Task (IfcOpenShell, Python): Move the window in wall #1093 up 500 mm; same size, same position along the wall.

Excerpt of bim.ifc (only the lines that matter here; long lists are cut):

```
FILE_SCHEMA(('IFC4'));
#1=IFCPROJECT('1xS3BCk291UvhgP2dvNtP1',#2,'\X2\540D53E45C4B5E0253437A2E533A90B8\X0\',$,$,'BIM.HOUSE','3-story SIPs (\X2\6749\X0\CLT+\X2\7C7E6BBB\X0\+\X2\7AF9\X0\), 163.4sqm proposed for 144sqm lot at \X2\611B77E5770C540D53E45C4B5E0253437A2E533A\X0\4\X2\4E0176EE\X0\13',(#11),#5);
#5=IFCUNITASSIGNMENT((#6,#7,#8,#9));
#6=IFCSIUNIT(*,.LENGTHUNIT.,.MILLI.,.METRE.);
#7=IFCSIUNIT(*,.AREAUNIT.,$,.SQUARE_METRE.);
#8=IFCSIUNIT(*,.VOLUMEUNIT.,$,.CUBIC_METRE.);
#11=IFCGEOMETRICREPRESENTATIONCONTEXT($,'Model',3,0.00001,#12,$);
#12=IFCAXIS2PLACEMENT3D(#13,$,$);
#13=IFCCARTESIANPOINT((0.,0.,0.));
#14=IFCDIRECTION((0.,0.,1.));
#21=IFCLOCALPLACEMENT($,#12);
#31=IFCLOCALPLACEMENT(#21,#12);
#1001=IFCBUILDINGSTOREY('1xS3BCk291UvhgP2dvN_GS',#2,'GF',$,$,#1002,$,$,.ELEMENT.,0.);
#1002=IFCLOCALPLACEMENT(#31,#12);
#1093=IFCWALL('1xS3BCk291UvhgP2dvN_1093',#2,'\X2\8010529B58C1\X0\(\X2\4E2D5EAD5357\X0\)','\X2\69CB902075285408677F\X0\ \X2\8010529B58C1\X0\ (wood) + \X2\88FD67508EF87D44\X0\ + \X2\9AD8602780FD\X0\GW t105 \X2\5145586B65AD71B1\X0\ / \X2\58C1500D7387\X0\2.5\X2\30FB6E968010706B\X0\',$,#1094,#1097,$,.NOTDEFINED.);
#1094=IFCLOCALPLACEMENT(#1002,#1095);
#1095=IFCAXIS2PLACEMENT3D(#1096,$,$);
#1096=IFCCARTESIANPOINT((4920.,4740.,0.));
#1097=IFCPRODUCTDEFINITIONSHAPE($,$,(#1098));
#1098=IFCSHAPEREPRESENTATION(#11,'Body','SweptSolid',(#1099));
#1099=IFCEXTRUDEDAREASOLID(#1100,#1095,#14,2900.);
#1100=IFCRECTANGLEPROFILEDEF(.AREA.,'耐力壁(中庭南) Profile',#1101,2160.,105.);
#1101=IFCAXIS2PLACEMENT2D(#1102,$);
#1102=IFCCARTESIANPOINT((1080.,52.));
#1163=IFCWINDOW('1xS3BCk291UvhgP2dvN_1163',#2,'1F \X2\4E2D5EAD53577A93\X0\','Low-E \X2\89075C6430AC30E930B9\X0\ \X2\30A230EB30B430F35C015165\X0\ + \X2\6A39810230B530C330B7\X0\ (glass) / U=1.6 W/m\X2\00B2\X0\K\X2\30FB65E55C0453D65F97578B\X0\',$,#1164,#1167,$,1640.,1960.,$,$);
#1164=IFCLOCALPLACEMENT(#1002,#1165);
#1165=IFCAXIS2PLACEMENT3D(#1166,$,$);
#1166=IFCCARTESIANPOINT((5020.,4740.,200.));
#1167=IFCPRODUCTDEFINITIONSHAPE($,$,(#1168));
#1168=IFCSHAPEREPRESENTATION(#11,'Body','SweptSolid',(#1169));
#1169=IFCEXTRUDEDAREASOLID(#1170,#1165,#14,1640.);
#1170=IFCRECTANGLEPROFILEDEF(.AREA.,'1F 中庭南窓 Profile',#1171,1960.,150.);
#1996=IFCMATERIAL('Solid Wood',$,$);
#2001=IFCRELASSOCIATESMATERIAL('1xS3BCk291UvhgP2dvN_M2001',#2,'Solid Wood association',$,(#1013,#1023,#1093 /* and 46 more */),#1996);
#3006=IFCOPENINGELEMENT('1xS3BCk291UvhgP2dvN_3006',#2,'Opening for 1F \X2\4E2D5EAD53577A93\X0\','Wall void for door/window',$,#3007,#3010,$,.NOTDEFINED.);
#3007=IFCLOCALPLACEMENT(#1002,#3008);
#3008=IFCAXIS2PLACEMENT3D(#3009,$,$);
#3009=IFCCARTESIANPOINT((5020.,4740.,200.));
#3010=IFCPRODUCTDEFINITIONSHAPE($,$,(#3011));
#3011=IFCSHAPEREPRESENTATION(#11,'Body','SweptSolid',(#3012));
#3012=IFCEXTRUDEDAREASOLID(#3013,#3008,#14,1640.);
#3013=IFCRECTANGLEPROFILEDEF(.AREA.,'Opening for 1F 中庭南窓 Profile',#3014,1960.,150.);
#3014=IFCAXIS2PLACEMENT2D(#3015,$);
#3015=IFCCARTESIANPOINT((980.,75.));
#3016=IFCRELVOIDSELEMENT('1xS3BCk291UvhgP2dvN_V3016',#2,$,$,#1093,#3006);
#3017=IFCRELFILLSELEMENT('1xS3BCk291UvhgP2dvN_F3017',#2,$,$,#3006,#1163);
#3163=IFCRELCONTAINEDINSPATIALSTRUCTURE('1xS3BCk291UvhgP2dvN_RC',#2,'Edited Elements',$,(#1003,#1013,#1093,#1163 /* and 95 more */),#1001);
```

```python
import numpy as np
import ifcopenshell
import ifcopenshell.api.geometry
import ifcopenshell.util.placement
import ifcopenshell.util.unit

model = ifcopenshell.open("bim.ifc")
unit_scale = ifcopenshell.util.unit.calculate_unit_scale(model)

window = model.by_guid("1xS3BCk291UvhgP2dvN_1163")
opening = window.FillsVoids[0].RelatingOpeningElement
dz = 500.0

shift = np.array([0.0, 0.0, dz])
# The window is not placed relative to its opening, so move both.
for product in (opening, window):
    matrix = ifcopenshell.util.placement.get_local_placement(product.ObjectPlacement)
    matrix[:3, 3] += shift
    ifcopenshell.api.geometry.edit_object_placement(model, product=product, matrix=matrix, is_si=False)

print(f"moved by {dz * unit_scale:+.3f} m")

model.write("bim_rev.ifc")
```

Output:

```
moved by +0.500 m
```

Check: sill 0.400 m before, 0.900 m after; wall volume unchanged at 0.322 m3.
